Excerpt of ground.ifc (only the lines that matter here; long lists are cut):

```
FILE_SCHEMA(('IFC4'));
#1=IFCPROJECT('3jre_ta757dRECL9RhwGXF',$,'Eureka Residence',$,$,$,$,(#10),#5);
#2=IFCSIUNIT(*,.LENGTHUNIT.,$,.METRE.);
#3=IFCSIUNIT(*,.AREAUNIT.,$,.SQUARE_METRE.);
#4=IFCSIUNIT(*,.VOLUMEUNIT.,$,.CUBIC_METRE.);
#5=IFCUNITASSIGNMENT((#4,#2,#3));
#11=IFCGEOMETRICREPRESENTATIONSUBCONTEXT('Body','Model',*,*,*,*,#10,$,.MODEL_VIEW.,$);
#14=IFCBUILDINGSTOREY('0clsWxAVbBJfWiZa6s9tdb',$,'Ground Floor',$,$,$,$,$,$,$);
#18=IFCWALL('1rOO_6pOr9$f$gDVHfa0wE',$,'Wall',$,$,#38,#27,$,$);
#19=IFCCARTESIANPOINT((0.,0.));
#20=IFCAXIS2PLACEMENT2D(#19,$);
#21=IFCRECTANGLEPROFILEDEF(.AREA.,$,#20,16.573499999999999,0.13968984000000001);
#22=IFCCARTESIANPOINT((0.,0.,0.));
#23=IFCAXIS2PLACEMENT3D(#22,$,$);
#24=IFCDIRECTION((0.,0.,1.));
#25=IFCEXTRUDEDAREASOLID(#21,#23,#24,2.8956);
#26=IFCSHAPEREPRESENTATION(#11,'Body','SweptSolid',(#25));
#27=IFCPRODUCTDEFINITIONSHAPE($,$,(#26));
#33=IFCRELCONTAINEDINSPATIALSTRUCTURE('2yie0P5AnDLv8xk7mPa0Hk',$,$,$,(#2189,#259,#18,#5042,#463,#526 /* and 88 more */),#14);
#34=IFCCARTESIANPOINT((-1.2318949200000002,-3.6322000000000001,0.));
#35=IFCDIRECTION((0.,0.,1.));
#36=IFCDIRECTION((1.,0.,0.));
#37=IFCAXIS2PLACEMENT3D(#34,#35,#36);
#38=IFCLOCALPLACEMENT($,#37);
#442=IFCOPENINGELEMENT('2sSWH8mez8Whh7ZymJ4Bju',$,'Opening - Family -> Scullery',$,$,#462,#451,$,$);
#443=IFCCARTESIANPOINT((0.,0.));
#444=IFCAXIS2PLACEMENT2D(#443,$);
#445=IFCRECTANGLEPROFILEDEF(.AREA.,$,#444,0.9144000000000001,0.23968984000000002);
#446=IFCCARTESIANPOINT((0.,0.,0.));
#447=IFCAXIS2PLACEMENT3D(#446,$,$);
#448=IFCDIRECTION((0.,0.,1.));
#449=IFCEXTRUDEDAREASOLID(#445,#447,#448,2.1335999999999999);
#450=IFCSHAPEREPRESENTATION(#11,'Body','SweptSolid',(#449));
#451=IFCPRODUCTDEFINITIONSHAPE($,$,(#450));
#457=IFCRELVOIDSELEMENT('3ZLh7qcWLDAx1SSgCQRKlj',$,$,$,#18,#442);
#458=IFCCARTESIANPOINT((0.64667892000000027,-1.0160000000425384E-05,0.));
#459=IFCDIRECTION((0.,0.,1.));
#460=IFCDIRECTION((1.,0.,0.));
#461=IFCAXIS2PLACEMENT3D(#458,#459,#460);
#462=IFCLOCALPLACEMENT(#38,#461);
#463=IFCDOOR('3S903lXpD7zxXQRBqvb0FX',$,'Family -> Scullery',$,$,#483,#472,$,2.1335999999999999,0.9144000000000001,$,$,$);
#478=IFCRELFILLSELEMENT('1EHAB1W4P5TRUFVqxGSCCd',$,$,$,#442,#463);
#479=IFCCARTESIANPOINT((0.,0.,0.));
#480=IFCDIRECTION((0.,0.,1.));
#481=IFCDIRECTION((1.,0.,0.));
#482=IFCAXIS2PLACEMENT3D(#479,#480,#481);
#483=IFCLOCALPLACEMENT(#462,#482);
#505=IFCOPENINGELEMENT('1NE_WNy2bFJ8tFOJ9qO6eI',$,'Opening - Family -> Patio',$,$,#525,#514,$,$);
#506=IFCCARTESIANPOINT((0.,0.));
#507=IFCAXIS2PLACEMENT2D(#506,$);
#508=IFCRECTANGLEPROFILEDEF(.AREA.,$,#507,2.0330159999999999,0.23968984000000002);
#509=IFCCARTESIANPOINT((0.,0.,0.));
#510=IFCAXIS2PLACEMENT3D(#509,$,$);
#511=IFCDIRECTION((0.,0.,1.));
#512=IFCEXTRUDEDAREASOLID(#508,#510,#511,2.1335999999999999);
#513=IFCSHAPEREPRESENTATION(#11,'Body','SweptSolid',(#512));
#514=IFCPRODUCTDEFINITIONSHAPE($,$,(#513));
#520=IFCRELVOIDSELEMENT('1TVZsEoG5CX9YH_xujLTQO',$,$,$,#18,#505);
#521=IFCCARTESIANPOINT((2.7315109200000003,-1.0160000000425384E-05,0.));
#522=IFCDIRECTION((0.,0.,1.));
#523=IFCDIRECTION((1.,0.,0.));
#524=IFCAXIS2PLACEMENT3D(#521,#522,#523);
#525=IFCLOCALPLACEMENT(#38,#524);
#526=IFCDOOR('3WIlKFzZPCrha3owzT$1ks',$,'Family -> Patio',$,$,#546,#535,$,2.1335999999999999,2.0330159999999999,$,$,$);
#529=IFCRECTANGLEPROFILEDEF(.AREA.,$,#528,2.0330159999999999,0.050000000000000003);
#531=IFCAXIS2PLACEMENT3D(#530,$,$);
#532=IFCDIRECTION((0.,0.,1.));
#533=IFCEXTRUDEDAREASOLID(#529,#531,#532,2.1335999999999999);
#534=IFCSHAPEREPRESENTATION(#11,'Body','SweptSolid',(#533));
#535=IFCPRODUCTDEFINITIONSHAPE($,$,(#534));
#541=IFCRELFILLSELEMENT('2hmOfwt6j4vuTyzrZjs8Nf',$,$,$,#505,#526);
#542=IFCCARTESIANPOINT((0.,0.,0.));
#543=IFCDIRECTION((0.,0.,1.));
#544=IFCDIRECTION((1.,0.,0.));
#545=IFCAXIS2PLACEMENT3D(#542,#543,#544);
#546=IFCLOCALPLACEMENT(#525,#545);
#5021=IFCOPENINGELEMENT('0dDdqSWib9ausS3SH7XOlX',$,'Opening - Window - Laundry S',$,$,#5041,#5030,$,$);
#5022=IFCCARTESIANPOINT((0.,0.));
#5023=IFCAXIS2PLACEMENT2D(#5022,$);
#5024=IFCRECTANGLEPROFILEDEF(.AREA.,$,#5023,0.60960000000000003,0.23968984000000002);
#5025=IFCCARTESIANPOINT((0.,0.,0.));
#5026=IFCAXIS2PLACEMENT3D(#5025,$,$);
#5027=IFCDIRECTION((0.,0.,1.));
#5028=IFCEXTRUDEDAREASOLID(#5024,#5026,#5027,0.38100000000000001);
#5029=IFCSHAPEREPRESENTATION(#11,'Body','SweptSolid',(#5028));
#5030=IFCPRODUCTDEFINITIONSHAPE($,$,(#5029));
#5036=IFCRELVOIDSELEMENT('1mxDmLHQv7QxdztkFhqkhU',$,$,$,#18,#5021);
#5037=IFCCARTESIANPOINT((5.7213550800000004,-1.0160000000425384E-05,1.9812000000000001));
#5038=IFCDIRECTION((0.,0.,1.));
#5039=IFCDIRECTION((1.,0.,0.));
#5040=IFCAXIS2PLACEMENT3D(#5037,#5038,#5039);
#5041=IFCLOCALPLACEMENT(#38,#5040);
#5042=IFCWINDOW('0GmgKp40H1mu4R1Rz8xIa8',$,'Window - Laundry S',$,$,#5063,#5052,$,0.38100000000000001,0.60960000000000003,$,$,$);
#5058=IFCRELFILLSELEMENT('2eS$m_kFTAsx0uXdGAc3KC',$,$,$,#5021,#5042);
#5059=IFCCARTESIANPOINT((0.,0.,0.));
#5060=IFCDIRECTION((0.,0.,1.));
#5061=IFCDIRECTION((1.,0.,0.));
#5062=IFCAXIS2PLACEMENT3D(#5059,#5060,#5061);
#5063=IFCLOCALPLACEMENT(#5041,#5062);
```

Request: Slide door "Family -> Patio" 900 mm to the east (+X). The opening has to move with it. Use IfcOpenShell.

```python
import ifcopenshell
import ifcopenshell.api.geometry
import ifcopenshell.util.placement

model = ifcopenshell.open("ground.ifc")

door = model.by_guid("3WIlKFzZPCrha3owzT$1ks")
opening = door.FillsVoids[0].RelatingOpeningElement
wall = opening.VoidsElements[0].RelatingBuildingElement

wall_matrix = ifcopenshell.util.placement.get_local_placement(wall.ObjectPlacement)
shift = wall_matrix[:3, 0] * 0.9
before = ifcopenshell.util.placement.get_local_placement(door.ObjectPlacement)[:3, 3].copy()

# The door is placed relative to its opening, so it follows when the opening moves.
matrix = ifcopenshell.util.placement.get_local_placement(opening.ObjectPlacement)
matrix[:3, 3] += shift
ifcopenshell.api.geometry.edit_object_placement(
    model, product=opening, matrix=matrix, is_si=False, should_transform_children=True
)

after = ifcopenshell.util.placement.get_local_placement(door.ObjectPlacement)[:3, 3]
print("door moved by", (after - before).round(3) + 0.0)

model.write("ground_updated.ifc")
```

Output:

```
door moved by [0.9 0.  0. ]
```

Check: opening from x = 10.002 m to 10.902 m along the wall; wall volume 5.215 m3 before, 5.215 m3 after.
